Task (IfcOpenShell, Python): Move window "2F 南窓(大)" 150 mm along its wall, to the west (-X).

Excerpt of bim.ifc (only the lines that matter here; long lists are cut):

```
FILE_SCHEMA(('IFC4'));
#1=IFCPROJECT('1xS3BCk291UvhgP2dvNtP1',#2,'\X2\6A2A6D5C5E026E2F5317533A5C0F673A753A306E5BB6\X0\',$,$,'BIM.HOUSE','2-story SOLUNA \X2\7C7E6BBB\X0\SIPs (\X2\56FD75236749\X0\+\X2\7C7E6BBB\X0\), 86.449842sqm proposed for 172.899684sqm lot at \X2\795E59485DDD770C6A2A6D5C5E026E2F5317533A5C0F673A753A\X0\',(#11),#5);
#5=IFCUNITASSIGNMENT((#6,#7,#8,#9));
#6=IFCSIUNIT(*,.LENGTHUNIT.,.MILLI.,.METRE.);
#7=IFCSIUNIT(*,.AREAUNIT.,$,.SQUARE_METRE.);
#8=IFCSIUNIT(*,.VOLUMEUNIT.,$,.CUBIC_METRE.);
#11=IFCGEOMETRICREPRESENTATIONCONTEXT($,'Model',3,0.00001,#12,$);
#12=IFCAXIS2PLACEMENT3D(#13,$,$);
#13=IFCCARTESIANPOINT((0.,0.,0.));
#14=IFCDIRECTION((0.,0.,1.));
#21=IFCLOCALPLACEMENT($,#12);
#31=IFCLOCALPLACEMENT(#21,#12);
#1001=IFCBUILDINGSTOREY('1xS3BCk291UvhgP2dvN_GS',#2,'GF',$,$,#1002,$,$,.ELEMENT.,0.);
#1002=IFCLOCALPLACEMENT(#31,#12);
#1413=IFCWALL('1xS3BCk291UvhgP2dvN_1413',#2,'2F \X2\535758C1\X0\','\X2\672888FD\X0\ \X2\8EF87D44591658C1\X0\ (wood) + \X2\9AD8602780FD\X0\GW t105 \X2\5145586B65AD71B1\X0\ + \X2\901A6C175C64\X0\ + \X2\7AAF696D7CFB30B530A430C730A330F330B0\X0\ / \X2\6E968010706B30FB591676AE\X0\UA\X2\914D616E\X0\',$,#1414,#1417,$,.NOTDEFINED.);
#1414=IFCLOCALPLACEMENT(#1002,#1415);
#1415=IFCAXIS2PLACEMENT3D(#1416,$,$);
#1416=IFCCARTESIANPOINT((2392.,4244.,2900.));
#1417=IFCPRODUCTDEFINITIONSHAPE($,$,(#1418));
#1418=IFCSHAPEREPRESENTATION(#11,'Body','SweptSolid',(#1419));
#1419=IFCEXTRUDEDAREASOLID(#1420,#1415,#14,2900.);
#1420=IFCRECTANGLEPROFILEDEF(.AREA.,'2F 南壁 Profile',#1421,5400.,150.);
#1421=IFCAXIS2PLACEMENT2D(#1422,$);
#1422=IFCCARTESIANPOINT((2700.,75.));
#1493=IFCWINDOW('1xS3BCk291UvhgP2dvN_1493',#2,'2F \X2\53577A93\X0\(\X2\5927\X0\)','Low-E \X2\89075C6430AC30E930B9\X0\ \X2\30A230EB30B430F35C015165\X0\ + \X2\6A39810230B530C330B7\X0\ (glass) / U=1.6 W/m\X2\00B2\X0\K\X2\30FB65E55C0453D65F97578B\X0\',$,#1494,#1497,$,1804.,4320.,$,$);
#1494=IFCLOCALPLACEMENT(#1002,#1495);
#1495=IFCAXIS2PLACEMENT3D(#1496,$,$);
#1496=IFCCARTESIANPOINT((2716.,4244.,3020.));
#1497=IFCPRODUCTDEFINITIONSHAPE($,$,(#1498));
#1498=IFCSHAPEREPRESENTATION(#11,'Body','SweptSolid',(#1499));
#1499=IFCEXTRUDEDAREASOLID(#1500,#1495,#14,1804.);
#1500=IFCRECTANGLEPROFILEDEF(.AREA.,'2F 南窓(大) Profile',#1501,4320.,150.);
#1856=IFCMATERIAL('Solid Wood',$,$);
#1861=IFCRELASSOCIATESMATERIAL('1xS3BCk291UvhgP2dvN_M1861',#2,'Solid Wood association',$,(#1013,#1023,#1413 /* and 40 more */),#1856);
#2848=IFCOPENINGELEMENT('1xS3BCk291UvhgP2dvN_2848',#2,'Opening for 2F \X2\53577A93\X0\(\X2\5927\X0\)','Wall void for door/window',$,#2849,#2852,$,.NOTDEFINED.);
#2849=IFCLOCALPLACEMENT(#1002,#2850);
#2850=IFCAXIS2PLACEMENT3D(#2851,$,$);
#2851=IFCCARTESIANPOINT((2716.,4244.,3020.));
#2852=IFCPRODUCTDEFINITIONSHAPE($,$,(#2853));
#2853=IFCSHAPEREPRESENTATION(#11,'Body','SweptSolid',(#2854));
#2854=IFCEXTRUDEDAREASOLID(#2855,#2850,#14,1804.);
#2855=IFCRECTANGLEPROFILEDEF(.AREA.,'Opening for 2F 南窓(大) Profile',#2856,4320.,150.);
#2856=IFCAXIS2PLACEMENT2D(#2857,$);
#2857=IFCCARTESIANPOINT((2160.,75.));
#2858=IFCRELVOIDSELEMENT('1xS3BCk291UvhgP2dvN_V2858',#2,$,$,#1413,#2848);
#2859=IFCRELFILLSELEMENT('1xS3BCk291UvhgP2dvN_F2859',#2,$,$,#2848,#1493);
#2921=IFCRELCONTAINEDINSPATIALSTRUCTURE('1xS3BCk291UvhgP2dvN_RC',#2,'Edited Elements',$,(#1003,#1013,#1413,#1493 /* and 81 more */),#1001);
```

```python
import ifcopenshell
import ifcopenshell.api.geometry
import ifcopenshell.util.placement

model = ifcopenshell.open("bim.ifc")

window = model.by_guid("1xS3BCk291UvhgP2dvN_1493")
opening = window.FillsVoids[0].RelatingOpeningElement
wall = opening.VoidsElements[0].RelatingBuildingElement

wall_matrix = ifcopenshell.util.placement.get_local_placement(wall.ObjectPlacement)
shift = wall_matrix[:3, 0] * -150.0
before = ifcopenshell.util.placement.get_local_placement(window.ObjectPlacement)[:3, 3].copy()

# The window is not placed relative to its opening, so move both.
for product in (opening, window):
    matrix = ifcopenshell.util.placement.get_local_placement(product.ObjectPlacement)
    matrix[:3, 3] += shift
    ifcopenshell.api.geometry.edit_object_placement(model, product=product, matrix=matrix, is_si=False)

after = ifcopenshell.util.placement.get_local_placement(window.ObjectPlacement)[:3, 3]
print("window moved by", (after - before).round(3) + 0.0)

model.write("bim_v2.ifc")
```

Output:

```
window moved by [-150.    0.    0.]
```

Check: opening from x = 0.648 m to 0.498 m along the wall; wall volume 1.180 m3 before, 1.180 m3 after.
